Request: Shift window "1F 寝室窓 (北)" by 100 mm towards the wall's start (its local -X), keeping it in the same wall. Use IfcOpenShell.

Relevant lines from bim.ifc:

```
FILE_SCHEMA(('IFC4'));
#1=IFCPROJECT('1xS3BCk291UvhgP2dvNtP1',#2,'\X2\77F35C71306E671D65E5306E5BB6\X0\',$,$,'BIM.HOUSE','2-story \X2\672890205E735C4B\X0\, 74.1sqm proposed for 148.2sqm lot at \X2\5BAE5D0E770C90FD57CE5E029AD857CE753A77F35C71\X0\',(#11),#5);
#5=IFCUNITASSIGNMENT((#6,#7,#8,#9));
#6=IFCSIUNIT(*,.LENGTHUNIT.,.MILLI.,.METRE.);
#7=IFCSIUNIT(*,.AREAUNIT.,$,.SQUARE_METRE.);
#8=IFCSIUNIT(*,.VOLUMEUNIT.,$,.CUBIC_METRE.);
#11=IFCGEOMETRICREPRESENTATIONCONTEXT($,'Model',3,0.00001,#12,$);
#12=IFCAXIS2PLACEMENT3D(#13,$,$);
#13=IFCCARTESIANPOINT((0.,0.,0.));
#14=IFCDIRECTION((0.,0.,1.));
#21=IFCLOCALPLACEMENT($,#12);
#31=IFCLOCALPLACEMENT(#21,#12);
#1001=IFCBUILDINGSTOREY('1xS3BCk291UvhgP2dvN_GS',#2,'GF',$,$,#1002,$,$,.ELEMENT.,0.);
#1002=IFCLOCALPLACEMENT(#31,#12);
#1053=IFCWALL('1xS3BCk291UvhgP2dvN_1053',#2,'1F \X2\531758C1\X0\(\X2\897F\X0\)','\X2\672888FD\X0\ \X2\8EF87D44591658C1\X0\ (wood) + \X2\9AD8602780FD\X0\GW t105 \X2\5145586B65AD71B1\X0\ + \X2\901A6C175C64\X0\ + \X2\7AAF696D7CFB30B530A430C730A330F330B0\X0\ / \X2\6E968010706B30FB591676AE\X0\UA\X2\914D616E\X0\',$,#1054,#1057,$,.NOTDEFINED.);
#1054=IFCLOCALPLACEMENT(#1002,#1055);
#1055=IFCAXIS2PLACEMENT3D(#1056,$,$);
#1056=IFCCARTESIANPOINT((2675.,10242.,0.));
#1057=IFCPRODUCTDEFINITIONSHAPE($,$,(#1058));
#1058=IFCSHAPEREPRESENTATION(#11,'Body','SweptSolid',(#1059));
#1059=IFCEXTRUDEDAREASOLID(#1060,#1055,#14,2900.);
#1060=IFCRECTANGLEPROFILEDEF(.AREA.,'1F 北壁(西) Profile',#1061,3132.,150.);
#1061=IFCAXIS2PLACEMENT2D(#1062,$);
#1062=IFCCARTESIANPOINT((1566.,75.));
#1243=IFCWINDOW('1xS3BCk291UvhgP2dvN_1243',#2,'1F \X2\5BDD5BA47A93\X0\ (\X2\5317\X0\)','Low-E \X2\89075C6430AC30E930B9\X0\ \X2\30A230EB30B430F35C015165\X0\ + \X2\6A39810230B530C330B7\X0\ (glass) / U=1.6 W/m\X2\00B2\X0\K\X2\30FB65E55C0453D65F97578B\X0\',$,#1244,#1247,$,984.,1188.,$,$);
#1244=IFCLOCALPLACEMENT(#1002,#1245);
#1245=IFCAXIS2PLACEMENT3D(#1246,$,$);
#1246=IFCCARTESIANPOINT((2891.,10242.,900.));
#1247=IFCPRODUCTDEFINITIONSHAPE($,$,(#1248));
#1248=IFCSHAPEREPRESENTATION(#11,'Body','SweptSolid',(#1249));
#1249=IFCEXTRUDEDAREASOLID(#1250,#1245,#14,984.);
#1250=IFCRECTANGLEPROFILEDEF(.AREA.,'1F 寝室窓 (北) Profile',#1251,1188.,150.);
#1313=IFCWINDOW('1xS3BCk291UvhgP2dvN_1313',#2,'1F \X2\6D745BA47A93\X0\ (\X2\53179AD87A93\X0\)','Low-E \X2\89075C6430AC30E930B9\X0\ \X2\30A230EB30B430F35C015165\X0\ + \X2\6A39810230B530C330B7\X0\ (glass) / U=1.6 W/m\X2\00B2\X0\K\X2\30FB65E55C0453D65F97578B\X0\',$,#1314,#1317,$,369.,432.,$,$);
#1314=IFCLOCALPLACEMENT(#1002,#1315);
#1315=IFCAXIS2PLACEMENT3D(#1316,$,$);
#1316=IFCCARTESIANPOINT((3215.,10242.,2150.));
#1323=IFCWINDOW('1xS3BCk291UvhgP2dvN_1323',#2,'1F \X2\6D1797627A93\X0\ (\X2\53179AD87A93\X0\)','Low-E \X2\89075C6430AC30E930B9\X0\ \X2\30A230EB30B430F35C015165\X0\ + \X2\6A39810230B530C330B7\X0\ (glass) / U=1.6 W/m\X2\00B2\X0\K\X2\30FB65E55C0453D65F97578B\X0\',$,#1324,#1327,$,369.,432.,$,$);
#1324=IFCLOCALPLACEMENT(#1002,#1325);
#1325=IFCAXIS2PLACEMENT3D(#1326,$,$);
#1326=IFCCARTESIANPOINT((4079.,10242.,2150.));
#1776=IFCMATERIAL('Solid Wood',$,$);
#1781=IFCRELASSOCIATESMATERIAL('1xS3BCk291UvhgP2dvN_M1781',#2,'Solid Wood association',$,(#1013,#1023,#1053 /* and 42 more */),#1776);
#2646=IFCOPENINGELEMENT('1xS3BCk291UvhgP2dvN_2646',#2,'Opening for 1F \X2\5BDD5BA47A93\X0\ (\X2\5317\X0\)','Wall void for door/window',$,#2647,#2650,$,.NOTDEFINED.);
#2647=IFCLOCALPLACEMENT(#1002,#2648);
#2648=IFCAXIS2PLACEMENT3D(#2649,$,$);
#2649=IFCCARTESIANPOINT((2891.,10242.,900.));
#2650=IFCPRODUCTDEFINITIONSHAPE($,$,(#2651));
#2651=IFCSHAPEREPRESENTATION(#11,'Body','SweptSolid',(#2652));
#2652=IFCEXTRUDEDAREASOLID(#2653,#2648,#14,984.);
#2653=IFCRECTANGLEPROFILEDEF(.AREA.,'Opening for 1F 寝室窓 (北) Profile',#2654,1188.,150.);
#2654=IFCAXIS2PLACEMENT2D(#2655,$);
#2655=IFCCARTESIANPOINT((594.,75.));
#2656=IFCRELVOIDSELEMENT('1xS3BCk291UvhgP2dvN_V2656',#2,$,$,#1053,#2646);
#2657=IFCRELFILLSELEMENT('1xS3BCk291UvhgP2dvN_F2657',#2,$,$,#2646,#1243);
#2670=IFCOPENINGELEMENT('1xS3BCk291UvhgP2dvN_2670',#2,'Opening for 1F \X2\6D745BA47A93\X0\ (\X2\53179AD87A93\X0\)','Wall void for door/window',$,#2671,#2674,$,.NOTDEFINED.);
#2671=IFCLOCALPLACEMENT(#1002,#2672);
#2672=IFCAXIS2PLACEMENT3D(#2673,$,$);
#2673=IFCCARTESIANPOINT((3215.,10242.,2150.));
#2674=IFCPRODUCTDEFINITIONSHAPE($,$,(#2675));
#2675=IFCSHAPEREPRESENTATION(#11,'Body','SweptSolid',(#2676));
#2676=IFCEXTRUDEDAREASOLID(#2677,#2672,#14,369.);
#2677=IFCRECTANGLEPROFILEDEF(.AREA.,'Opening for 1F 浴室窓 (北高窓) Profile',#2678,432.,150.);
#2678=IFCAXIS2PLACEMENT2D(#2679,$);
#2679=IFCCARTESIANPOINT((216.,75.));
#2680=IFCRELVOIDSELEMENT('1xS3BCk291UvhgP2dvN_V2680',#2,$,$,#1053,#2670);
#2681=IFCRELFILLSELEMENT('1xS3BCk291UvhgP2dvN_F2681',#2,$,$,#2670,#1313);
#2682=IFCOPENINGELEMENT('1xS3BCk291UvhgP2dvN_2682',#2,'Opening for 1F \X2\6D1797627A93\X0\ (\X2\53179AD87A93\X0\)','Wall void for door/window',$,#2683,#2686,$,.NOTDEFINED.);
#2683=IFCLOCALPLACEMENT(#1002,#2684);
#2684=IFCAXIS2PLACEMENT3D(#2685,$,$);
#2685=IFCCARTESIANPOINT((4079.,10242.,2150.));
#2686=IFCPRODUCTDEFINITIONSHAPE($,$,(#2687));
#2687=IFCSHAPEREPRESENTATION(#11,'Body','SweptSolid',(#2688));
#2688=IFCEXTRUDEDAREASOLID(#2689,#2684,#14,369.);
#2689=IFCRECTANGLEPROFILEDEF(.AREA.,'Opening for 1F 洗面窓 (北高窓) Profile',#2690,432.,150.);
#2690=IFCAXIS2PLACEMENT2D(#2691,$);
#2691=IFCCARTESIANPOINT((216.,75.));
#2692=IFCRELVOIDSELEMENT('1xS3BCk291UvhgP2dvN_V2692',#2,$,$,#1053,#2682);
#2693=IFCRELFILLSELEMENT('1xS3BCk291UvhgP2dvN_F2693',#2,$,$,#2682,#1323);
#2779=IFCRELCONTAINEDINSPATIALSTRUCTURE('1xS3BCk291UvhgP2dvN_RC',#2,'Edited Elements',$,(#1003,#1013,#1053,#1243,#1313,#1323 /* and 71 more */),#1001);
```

```python
import ifcopenshell
import ifcopenshell.api.geometry
import ifcopenshell.util.placement
import ifcopenshell.util.unit

model = ifcopenshell.open("bim.ifc")
unit_scale = ifcopenshell.util.unit.calculate_unit_scale(model)

window = model.by_guid("1xS3BCk291UvhgP2dvN_1243")
opening = window.FillsVoids[0].RelatingOpeningElement
wall = opening.VoidsElements[0].RelatingBuildingElement

wall_matrix = ifcopenshell.util.placement.get_local_placement(wall.ObjectPlacement)
shift = wall_matrix[:3, 0] * -0.1 / unit_scale
before = ifcopenshell.util.placement.get_local_placement(window.ObjectPlacement)[:3, 3].copy()

# The window is not placed relative to its opening, so move both.
for product in (opening, window):
    matrix = ifcopenshell.util.placement.get_local_placement(product.ObjectPlacement)
    matrix[:3, 3] += shift
    ifcopenshell.api.geometry.edit_object_placement(model, product=product, matrix=matrix, is_si=False)

after = ifcopenshell.util.placement.get_local_placement(window.ObjectPlacement)[:3, 3]
print("window moved by", (after - before).round(3) + 0.0)

model.write("bim_v2.ifc")
```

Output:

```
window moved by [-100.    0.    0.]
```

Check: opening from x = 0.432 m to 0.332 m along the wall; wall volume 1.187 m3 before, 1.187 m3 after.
